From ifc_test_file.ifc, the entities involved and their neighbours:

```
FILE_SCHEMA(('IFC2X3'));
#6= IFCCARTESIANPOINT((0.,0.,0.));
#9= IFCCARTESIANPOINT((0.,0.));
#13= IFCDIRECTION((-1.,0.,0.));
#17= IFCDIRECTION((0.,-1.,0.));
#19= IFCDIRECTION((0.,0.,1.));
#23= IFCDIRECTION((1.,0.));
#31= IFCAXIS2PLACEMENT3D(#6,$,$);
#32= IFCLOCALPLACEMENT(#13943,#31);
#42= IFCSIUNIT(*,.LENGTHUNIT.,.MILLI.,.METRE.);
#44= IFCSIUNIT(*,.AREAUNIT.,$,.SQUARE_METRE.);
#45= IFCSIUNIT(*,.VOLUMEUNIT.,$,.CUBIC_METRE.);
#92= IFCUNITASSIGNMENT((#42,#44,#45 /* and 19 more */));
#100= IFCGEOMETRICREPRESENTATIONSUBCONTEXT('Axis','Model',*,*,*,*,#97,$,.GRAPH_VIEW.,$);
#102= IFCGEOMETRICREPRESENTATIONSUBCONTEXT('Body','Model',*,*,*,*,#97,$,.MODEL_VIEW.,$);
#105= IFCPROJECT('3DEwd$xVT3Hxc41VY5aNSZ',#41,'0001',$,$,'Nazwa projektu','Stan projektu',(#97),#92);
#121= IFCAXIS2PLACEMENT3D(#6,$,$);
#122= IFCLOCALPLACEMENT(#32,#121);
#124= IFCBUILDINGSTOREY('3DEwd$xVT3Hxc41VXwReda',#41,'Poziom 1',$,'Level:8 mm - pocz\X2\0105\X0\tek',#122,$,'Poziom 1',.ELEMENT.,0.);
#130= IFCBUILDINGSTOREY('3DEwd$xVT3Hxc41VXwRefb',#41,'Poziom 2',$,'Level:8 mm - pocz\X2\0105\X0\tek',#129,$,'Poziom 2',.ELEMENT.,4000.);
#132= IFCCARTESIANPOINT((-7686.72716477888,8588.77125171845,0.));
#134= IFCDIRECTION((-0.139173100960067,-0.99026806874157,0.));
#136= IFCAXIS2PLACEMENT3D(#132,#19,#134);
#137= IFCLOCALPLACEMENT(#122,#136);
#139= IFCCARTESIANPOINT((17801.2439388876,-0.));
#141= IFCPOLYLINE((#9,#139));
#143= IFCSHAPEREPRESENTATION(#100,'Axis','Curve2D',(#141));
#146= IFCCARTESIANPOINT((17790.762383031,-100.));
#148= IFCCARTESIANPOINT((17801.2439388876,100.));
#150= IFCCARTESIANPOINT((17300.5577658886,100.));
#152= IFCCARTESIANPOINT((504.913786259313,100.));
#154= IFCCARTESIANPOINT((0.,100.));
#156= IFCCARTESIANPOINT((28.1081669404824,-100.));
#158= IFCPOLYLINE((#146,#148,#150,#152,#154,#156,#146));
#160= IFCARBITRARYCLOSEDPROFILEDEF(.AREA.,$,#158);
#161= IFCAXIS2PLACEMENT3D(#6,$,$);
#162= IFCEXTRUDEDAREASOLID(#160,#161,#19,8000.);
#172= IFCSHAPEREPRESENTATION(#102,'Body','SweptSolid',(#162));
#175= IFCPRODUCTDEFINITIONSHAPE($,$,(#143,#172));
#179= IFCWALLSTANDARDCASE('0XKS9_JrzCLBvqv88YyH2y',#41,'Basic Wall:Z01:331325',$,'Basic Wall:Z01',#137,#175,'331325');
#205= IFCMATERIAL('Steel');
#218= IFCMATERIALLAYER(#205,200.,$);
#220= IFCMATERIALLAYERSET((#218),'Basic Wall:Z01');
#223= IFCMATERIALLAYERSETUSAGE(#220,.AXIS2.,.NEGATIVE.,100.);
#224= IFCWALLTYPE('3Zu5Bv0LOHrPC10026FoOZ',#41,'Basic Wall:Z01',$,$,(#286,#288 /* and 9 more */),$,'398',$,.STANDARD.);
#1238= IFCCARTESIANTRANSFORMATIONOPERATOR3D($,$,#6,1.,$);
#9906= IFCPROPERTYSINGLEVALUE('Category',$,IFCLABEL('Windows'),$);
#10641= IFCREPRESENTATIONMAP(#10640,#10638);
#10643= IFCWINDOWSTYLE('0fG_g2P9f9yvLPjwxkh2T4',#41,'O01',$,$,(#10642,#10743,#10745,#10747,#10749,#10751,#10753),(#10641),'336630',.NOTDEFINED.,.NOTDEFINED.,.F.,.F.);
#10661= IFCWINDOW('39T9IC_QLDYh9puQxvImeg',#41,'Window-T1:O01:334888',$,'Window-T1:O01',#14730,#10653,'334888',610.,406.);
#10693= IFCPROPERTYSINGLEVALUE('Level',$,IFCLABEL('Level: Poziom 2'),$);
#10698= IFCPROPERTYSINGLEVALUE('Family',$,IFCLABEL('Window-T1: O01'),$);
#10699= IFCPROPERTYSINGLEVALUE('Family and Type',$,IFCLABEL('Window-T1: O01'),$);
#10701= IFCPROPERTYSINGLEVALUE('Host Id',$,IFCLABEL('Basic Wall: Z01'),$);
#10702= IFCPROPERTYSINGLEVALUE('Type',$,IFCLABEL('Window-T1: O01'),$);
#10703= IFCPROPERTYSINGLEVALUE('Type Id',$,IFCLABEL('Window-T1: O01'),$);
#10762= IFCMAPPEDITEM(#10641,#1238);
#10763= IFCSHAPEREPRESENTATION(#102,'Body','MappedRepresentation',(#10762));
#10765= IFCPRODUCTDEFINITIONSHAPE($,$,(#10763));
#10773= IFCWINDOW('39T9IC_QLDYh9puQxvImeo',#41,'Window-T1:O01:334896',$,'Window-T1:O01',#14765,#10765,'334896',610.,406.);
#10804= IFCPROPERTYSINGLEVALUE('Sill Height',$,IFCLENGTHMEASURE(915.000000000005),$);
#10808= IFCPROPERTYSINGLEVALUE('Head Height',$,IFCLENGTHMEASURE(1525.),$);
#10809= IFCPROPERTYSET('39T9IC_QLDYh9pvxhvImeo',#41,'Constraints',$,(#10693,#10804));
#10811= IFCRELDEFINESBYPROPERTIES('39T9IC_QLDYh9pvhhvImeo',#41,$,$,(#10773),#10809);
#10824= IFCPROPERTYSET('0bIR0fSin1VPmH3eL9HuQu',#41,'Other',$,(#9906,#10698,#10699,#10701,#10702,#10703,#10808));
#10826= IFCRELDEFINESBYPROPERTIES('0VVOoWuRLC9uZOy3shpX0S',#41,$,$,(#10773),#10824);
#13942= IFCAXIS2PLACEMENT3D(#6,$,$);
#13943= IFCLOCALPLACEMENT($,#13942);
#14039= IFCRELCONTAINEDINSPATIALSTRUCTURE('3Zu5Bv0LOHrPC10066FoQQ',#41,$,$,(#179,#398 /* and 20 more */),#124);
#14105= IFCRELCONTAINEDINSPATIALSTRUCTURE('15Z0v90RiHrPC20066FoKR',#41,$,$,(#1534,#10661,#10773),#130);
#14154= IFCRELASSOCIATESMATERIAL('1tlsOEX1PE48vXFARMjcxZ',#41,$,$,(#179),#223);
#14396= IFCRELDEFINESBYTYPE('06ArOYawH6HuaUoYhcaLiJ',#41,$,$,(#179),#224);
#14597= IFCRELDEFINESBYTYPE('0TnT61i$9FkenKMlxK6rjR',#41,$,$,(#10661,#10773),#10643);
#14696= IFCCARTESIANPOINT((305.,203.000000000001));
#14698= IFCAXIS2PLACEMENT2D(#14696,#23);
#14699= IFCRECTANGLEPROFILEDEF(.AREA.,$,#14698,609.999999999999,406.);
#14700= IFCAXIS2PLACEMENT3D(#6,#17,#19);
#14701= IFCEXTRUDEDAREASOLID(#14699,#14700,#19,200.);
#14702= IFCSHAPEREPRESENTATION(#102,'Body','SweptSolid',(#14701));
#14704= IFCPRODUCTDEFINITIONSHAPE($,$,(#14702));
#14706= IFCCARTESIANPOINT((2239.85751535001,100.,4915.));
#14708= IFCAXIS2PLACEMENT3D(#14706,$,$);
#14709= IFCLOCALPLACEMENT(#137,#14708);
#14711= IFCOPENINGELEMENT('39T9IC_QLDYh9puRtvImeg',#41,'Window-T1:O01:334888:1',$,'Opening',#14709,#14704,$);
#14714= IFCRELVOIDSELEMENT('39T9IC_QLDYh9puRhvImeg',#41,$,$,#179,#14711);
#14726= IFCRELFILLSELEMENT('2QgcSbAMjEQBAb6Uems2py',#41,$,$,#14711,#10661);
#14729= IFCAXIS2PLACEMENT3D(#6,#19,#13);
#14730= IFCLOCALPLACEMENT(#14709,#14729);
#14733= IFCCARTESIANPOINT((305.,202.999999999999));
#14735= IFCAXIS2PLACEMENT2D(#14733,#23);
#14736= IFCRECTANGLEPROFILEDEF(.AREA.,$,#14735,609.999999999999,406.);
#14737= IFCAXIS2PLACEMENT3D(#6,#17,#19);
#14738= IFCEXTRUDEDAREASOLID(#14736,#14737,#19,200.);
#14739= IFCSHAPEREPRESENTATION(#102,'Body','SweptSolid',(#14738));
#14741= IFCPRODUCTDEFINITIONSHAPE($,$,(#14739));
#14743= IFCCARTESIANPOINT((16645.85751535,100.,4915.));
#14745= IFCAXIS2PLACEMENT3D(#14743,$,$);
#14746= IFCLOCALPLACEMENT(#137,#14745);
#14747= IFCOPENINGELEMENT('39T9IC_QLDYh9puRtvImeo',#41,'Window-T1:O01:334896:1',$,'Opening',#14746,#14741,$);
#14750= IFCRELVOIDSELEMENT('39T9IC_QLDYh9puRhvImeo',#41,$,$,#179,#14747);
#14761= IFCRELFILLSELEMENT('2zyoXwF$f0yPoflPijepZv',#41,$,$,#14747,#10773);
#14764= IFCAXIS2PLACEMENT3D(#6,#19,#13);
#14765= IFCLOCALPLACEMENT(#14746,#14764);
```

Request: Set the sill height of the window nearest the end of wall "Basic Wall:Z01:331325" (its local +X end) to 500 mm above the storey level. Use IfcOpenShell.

```python
import numpy as np
import ifcopenshell
import ifcopenshell.api.geometry
import ifcopenshell.api.pset
import ifcopenshell.geom
import ifcopenshell.util.element
import ifcopenshell.util.placement
import ifcopenshell.util.shape
import ifcopenshell.util.unit

model = ifcopenshell.open("ifc_test_file.ifc")
unit_scale = ifcopenshell.util.unit.calculate_unit_scale(model)

window = model.by_id(10773)
opening = window.FillsVoids[0].RelatingOpeningElement
storey = ifcopenshell.util.element.get_container(window, ifc_class="IfcBuildingStorey")
level = ifcopenshell.util.placement.get_local_placement(storey.ObjectPlacement)[2, 3]

# The opening's origin need not be at the sill, so measure its lowest point.
shape = ifcopenshell.geom.create_shape(ifcopenshell.geom.settings(), opening)
bottom = ifcopenshell.util.shape.get_shape_bottom_elevation(shape, shape.geometry) / unit_scale
dz = level + 0.5 / unit_scale - bottom

shift = np.array([0.0, 0.0, dz])
# The window is placed relative to its opening, so it follows when the opening moves.
matrix = ifcopenshell.util.placement.get_local_placement(opening.ObjectPlacement)
matrix[:3, 3] += shift
ifcopenshell.api.geometry.edit_object_placement(
    model, product=opening, matrix=matrix, is_si=False, should_transform_children=True
)

# Keep the stored heights in step.
pset = model.by_id(ifcopenshell.util.element.get_pset(window, "Constraints", should_inherit=False)["id"])
ifcopenshell.api.pset.edit_pset(model, pset=pset, properties={
    "Sill Height": model.create_entity("IfcLengthMeasure", ifcopenshell.util.element.get_pset(window, "Constraints", "Sill Height") + dz),
})
pset = model.by_id(ifcopenshell.util.element.get_pset(window, "Other", should_inherit=False)["id"])
ifcopenshell.api.pset.edit_pset(model, pset=pset, properties={
    "Head Height": model.create_entity("IfcLengthMeasure", ifcopenshell.util.element.get_pset(window, "Other", "Head Height") + dz),
})

print(f"moved by {dz * unit_scale:+.3f} m")

model.write("ifc_test_file_edited.ifc")
```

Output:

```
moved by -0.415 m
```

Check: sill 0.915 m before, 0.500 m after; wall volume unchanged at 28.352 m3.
